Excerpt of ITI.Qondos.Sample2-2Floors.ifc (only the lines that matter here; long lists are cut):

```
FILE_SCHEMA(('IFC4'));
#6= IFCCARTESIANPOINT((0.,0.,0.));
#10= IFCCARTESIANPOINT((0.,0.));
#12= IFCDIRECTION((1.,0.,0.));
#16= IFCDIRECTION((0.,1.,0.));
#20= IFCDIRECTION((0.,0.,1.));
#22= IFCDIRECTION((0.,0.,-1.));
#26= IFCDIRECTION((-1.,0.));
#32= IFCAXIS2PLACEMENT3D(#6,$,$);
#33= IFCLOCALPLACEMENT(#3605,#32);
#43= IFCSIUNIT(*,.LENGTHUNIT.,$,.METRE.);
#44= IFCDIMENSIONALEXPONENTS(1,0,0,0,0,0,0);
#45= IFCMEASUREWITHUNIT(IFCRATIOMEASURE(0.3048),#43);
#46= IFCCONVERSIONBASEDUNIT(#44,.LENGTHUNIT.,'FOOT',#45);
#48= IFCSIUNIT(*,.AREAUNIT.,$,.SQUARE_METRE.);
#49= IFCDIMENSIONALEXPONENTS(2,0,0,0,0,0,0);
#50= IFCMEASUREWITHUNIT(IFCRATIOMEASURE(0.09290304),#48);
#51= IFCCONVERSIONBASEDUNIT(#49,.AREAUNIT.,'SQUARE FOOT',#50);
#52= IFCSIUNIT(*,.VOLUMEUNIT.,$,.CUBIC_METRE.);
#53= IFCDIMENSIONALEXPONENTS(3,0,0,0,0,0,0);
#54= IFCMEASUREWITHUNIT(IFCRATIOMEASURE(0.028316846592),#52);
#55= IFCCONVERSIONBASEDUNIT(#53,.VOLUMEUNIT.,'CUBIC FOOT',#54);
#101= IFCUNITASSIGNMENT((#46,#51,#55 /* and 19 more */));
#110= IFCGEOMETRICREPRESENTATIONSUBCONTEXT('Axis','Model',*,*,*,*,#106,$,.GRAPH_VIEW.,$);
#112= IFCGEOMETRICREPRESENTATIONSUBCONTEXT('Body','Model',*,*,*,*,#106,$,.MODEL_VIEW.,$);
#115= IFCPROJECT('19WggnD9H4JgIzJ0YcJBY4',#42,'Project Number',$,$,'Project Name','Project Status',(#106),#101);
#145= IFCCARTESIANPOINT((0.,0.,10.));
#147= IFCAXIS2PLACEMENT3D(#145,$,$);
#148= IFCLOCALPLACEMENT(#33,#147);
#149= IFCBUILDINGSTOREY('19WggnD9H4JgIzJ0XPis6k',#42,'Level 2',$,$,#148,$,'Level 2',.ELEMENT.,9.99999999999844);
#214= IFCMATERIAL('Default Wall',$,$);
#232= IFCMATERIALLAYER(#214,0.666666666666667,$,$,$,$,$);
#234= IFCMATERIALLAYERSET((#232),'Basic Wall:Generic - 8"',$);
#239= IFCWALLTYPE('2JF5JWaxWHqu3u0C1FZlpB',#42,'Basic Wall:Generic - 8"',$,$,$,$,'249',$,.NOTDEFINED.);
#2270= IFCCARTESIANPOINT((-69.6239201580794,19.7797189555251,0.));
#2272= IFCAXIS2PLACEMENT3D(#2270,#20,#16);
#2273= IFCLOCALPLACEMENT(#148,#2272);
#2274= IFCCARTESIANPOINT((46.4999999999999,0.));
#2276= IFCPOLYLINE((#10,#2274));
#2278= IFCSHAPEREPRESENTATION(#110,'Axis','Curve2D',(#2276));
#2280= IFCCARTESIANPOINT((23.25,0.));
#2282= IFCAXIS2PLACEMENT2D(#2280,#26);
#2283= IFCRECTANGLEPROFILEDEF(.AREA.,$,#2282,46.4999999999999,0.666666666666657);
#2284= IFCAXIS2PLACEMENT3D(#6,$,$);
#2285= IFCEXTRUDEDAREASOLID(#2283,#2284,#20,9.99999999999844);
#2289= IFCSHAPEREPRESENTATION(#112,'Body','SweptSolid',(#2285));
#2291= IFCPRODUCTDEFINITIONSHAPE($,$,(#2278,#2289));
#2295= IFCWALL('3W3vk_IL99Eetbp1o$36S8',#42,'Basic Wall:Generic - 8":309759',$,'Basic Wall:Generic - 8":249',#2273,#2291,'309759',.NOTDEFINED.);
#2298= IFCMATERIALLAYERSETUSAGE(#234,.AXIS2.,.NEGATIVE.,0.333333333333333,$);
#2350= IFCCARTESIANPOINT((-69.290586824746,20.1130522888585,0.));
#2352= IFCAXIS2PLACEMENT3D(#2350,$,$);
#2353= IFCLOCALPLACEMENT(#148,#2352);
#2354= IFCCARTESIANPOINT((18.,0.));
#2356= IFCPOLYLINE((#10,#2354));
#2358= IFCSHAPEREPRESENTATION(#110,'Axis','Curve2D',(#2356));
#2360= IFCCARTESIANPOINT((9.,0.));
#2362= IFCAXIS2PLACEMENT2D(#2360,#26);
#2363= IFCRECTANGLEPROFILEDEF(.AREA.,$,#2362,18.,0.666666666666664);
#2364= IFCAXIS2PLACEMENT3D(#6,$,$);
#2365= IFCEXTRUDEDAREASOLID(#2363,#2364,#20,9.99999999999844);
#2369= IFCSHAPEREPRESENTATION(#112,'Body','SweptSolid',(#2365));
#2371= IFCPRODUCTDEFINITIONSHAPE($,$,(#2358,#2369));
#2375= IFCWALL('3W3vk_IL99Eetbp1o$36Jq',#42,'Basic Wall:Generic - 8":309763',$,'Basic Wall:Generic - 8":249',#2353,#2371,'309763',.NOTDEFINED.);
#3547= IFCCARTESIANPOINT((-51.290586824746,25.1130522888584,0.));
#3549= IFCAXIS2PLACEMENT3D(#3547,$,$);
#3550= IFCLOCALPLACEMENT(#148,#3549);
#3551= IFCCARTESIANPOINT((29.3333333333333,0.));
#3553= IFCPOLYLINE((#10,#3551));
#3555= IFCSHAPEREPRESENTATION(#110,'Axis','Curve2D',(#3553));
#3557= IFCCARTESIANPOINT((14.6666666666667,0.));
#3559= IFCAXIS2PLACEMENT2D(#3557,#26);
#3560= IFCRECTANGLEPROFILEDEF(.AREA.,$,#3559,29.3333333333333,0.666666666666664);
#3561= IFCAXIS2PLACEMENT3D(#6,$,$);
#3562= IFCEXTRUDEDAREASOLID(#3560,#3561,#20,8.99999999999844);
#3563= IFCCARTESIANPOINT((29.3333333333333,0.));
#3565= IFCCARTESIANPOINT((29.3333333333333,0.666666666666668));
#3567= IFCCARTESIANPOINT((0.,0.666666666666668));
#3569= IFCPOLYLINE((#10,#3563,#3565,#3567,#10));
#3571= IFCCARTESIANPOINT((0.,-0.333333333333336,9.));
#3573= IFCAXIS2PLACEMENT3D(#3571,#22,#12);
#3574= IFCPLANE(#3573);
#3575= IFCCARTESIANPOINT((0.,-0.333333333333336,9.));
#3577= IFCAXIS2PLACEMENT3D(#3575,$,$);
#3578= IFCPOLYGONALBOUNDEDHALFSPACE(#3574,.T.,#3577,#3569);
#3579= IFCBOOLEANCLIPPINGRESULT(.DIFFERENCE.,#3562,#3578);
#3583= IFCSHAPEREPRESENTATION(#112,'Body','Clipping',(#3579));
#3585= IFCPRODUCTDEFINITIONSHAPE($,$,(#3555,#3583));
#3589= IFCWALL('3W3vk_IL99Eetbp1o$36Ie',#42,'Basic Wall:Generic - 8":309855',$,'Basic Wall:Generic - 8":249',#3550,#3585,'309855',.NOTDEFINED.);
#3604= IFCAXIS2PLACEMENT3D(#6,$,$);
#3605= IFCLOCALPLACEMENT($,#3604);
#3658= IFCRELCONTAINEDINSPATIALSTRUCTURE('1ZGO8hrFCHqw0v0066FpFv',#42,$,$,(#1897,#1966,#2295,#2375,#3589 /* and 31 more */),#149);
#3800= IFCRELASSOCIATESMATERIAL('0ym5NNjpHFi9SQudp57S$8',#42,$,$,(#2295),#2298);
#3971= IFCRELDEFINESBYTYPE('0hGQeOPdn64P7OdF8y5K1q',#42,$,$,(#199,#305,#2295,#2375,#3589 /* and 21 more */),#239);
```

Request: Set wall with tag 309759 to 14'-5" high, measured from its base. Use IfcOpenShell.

```python
import ifcopenshell
import ifcopenshell.geom
import ifcopenshell.util.representation
import ifcopenshell.util.shape
import ifcopenshell.util.unit

model = ifcopenshell.open("ITI.Qondos.Sample2-2Floors.ifc")
unit_scale = ifcopenshell.util.unit.calculate_unit_scale(model)
settings = ifcopenshell.geom.settings()


def volume(element):
    """Net volume in cubic metres, openings subtracted."""
    shape = ifcopenshell.geom.create_shape(settings, element)
    return ifcopenshell.util.shape.get_volume(shape.geometry)


wall = model.by_guid("3W3vk_IL99Eetbp1o$36S8")
before = volume(wall)

body = ifcopenshell.util.representation.get_representation(wall, "Model", "Body")
solid = body.Items[0]
old_height = solid.Depth
solid.Depth = 173 * 0.0254 / unit_scale
after = volume(wall)

print(f"height {old_height:g} -> {solid.Depth:g}, volume {before:.3f} -> {after:.3f} m3")

model.write("ITI.Qondos.Sample2-2Floors_rev.ifc")
```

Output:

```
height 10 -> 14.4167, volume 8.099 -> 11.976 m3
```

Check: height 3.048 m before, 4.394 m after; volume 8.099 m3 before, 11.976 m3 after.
